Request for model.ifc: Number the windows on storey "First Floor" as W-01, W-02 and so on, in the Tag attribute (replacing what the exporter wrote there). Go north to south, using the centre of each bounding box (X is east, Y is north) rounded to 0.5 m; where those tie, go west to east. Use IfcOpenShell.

First a look at what the model holds.

```python
import ifcopenshell
import ifcopenshell.util.element
import ifcopenshell.util.placement

model = ifcopenshell.open("model.ifc")
print(model.schema)
storey = next(s for s in model.by_type("IfcBuildingStorey") if s.Name == "First Floor")
windows = [e for e in ifcopenshell.util.element.get_decomposition(storey) if e.is_a("IfcWindow")]
for e in sorted(windows, key=lambda e: e.id()):
    origin = ifcopenshell.util.placement.get_local_placement(e.ObjectPlacement)[:3, 3]
    print(e.id(), e.Tag, e.Name, origin.round(2) + 0.0, sep=" | ")
```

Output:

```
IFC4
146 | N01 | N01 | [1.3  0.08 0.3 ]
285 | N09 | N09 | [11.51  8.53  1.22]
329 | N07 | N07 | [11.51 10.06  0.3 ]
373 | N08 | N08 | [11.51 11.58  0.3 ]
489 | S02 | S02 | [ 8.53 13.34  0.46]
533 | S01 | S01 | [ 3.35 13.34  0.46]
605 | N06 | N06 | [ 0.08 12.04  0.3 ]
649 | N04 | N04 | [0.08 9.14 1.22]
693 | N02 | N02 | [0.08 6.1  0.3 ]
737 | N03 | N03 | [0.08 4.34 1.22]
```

```python
import ifcopenshell
import ifcopenshell.geom
import ifcopenshell.util.element
import ifcopenshell.util.shape

model = ifcopenshell.open("model.ifc")
settings = ifcopenshell.geom.settings()
settings.set("use-world-coords", True)


def centre(element):
    shape = ifcopenshell.geom.create_shape(settings, element)
    return ifcopenshell.util.shape.get_bbox_centroid(shape.geometry)


storey = next(s for s in model.by_type("IfcBuildingStorey") if s.Name == "First Floor")
windows = [e for e in ifcopenshell.util.element.get_decomposition(storey) if e.is_a("IfcWindow")]

# Insertion points can sit at a corner or the storey origin, so sort by the geometry (in metres).
centres = {e: centre(e) for e in windows}
windows.sort(key=lambda e: (-round(centres[e][1] / 0.5), centres[e][0]))

for i, e in enumerate(windows, start=1):
    number = f"W-{i:02d}"
    e.Tag = number
    print(e.id(), number)

model.write("model_v2.ifc")
```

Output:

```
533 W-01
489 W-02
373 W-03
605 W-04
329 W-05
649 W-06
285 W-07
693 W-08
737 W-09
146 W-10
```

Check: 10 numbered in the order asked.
